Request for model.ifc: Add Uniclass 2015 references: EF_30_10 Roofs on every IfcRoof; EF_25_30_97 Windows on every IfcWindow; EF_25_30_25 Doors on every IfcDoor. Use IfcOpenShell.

First a look at what the model holds.

```python
import ifcopenshell

model = ifcopenshell.open("model.ifc")
print(model.schema)
print("classifications:", [c.Name for c in model.by_type("IfcClassification")])
for ifc_class in ("IfcDoor", "IfcRoof", "IfcStair", "IfcWall", "IfcWindow"):
    print(ifc_class, len(model.by_type(ifc_class)))
```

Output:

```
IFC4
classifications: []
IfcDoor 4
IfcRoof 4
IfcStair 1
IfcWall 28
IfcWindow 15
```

```python
import ifcopenshell
import ifcopenshell.api.classification

model = ifcopenshell.open("model.ifc")

system = ifcopenshell.api.classification.add_classification(model, classification="Uniclass 2015")

codes = {
    "IfcRoof": ("EF_30_10", "Roofs"),
    "IfcWindow": ("EF_25_30_97", "Windows"),
    "IfcDoor": ("EF_25_30_25", "Doors"),
}
for ifc_class, (code, name) in codes.items():
    products = model.by_type(ifc_class)
    ifcopenshell.api.classification.add_reference(
        model, products=products, classification=system, identification=code, name=name
    )
    print(code, len(products))

model.write("model_edited.ifc")
```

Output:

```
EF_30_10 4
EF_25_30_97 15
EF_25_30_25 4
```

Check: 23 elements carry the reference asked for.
